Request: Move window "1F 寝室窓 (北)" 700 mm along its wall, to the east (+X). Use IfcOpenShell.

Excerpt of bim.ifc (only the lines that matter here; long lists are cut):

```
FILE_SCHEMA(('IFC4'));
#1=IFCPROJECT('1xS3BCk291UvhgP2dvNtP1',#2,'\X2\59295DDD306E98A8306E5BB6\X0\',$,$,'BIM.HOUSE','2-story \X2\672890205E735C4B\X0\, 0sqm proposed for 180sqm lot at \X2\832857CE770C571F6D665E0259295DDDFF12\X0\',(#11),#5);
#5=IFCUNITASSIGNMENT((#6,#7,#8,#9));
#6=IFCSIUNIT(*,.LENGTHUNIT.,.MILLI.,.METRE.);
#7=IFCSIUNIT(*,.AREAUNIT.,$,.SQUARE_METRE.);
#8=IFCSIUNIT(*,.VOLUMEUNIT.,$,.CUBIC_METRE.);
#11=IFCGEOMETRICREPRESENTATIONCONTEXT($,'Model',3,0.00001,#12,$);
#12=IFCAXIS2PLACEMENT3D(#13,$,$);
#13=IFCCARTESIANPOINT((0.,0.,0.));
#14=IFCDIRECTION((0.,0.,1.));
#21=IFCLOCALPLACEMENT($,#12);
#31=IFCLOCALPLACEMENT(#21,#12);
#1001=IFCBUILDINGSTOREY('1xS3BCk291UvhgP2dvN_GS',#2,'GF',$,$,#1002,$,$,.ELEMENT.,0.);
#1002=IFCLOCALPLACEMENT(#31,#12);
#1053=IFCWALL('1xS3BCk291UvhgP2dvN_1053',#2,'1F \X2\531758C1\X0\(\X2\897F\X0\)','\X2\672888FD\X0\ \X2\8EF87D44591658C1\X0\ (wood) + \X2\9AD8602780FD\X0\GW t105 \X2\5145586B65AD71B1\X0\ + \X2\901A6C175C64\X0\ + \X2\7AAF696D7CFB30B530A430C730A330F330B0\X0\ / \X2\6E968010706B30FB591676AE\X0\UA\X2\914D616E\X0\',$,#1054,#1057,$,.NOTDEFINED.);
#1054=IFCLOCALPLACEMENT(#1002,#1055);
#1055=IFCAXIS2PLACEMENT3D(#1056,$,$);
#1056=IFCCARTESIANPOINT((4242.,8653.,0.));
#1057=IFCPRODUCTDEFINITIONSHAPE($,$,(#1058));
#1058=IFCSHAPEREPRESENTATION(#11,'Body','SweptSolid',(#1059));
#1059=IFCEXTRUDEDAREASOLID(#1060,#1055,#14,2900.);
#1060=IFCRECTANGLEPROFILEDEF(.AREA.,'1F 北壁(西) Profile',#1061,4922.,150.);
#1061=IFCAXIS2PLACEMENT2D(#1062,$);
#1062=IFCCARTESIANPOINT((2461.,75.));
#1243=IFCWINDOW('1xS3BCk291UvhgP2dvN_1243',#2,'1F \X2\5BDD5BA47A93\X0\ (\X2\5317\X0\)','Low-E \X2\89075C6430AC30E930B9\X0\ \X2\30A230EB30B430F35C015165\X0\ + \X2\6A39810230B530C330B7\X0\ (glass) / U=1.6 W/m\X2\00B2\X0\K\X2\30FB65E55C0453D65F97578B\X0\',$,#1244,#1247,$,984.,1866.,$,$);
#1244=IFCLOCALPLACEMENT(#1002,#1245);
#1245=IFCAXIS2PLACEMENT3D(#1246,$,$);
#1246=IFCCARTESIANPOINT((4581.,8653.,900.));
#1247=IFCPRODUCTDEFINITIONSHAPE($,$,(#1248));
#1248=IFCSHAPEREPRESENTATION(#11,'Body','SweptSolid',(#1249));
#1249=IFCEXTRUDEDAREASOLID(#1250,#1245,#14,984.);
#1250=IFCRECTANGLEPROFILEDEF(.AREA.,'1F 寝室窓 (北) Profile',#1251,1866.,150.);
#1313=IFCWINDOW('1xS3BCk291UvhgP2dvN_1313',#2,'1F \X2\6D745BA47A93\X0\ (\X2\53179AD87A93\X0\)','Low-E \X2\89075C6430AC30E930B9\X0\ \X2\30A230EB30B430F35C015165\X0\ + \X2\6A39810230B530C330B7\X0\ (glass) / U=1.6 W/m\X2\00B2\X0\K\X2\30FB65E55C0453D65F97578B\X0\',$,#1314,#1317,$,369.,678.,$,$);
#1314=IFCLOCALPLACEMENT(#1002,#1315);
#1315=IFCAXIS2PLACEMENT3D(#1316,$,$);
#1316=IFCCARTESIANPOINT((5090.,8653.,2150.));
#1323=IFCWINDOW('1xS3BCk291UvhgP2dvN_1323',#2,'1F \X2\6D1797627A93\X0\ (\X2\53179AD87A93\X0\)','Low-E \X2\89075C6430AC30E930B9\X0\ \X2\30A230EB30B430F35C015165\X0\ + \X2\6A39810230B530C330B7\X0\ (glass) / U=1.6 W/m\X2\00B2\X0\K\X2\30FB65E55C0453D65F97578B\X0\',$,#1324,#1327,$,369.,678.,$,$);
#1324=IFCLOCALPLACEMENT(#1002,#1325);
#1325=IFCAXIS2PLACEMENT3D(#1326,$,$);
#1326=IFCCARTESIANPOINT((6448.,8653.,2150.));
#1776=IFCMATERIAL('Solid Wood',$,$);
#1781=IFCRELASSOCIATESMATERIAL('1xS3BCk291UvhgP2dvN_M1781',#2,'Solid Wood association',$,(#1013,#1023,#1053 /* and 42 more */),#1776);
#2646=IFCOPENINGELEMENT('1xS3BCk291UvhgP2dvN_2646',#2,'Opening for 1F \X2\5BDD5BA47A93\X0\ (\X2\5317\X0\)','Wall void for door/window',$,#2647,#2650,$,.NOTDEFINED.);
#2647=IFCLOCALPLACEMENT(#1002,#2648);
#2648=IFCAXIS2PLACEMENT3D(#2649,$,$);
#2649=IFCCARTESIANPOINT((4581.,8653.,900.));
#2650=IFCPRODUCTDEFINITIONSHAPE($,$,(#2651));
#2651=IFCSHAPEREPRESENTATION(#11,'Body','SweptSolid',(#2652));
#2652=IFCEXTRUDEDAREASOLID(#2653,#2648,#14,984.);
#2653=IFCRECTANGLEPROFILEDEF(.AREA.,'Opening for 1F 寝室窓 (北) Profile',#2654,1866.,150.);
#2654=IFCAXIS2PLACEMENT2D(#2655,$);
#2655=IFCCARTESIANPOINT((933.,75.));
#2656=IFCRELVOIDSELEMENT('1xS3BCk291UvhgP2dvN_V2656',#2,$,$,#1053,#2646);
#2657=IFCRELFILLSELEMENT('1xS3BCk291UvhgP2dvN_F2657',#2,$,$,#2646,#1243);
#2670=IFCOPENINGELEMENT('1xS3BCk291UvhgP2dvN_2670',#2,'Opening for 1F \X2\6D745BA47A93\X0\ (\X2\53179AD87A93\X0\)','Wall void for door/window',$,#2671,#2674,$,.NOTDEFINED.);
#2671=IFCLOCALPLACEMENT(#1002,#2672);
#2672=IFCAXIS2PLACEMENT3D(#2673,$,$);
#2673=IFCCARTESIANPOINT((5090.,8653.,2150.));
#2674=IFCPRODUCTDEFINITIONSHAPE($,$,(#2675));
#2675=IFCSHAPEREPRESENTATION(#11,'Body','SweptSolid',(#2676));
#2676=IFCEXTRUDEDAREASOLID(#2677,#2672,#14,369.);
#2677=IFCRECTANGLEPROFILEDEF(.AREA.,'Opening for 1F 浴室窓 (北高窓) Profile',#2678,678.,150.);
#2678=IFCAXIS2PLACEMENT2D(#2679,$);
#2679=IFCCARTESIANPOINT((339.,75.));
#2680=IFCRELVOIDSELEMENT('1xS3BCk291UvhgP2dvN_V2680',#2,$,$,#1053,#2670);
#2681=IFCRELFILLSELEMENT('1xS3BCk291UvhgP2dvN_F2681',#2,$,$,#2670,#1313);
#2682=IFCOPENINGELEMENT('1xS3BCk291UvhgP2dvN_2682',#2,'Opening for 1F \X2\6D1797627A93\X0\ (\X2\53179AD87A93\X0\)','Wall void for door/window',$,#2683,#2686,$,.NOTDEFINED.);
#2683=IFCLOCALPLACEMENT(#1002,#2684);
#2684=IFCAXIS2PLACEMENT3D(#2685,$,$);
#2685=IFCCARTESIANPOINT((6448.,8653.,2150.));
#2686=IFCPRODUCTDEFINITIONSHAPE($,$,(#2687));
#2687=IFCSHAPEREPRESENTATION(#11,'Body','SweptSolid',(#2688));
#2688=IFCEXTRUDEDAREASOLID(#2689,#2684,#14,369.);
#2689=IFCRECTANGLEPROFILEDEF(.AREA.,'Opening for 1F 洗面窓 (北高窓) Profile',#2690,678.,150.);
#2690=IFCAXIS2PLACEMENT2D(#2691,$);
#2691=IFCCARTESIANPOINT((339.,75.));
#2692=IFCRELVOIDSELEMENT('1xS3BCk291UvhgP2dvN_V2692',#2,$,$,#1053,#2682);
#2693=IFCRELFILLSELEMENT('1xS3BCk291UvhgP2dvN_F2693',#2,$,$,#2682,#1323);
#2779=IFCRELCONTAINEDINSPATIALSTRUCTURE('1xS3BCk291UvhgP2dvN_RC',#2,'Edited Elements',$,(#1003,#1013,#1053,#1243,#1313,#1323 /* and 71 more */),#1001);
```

```python
import ifcopenshell
import ifcopenshell.api.geometry
import ifcopenshell.util.placement

model = ifcopenshell.open("bim.ifc")

window = model.by_guid("1xS3BCk291UvhgP2dvN_1243")
opening = window.FillsVoids[0].RelatingOpeningElement
wall = opening.VoidsElements[0].RelatingBuildingElement

wall_matrix = ifcopenshell.util.placement.get_local_placement(wall.ObjectPlacement)
shift = wall_matrix[:3, 0] * 700.0
before = ifcopenshell.util.placement.get_local_placement(window.ObjectPlacement)[:3, 3].copy()

# The window is not placed relative to its opening, so move both.
for product in (opening, window):
    matrix = ifcopenshell.util.placement.get_local_placement(product.ObjectPlacement)
    matrix[:3, 3] += shift
    ifcopenshell.api.geometry.edit_object_placement(model, product=product, matrix=matrix, is_si=False)

after = ifcopenshell.util.placement.get_local_placement(window.ObjectPlacement)[:3, 3]
print("window moved by", (after - before).round(3) + 0.0)

model.write("bim_updated.ifc")
```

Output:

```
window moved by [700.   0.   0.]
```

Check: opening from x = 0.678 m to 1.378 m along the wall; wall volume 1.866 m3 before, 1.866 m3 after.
